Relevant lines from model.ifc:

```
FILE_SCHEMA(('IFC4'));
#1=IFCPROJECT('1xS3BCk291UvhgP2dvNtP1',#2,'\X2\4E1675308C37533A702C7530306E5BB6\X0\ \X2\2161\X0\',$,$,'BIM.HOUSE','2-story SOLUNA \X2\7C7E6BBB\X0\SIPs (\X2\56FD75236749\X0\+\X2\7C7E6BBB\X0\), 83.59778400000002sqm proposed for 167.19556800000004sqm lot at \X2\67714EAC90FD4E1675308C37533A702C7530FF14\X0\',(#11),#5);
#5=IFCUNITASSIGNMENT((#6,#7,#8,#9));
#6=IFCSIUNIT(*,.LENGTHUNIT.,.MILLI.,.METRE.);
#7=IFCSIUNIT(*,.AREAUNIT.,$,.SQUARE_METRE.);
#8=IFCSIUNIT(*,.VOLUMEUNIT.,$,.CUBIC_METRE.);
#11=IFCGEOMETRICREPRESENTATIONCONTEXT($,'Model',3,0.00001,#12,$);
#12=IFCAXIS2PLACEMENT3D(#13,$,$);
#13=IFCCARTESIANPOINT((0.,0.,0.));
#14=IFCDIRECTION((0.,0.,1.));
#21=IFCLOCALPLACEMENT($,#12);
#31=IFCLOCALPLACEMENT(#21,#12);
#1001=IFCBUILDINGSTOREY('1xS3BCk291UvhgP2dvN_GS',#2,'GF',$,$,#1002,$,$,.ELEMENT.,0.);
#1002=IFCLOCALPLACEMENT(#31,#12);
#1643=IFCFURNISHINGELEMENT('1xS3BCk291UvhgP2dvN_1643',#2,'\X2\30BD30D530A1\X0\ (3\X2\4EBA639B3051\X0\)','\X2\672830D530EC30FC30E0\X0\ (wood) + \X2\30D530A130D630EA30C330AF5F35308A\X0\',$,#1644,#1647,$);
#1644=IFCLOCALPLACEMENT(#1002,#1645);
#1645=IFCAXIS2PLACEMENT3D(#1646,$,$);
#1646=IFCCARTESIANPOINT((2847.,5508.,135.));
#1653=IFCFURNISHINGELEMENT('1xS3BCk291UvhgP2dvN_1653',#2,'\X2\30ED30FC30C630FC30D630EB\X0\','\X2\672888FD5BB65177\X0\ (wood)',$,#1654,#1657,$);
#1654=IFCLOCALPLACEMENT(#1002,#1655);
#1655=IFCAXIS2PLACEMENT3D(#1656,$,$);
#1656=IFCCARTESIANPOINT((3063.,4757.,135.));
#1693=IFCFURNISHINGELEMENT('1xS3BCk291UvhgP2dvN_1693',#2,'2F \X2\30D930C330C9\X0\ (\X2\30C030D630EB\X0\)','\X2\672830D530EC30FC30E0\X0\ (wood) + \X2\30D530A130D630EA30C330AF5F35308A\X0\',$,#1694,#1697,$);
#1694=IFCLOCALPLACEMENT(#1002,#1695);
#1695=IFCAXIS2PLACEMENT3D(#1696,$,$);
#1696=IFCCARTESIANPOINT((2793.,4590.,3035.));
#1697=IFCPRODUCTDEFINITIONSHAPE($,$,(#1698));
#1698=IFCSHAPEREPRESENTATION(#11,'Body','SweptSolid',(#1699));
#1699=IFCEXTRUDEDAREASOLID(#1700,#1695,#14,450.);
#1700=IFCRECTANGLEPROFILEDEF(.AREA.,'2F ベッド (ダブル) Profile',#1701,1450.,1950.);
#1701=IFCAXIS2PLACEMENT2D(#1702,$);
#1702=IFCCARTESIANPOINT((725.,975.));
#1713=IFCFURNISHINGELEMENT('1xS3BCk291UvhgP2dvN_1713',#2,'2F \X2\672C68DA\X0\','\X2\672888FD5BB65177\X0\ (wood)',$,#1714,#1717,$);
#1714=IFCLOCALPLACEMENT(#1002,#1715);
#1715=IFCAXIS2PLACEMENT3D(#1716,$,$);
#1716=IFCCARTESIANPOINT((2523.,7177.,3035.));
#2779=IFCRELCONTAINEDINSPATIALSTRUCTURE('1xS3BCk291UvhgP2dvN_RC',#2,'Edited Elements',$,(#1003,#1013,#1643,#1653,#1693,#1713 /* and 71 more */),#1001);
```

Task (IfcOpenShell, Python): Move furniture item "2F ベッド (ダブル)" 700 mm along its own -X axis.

```python
import ifcopenshell
import ifcopenshell.api.geometry
import ifcopenshell.util.placement

model = ifcopenshell.open("model.ifc")

item = model.by_id(1693)
matrix = ifcopenshell.util.placement.get_local_placement(item.ObjectPlacement)
matrix[:3, 3] -= matrix[:3, 0] * 700.0
ifcopenshell.api.geometry.edit_object_placement(model, product=item, matrix=matrix, is_si=False)

print(ifcopenshell.util.placement.get_local_placement(item.ObjectPlacement).round(3) + 0.0)

model.write("model_updated.ifc")
```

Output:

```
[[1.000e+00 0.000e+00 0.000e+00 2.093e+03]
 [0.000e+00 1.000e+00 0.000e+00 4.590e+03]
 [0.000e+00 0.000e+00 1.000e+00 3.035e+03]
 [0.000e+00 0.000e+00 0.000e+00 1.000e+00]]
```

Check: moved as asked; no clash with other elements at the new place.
